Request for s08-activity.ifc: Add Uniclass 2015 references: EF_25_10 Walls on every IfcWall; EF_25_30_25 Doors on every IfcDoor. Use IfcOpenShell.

First a look at what the model holds.

```python
import ifcopenshell

model = ifcopenshell.open("s08-activity.ifc")
print(model.schema)
print("classifications:", [c.Name for c in model.by_type("IfcClassification")])
for ifc_class in ("IfcDoor", "IfcRoof", "IfcStair", "IfcWall", "IfcWindow"):
    print(ifc_class, len(model.by_type(ifc_class)))
```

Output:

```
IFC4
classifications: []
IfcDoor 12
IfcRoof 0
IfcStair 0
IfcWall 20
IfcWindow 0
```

```python
import ifcopenshell
import ifcopenshell.api.classification

model = ifcopenshell.open("s08-activity.ifc")

system = ifcopenshell.api.classification.add_classification(model, classification="Uniclass 2015")

codes = {
    "IfcWall": ("EF_25_10", "Walls"),
    "IfcDoor": ("EF_25_30_25", "Doors"),
}
for ifc_class, (code, name) in codes.items():
    products = model.by_type(ifc_class)
    ifcopenshell.api.classification.add_reference(
        model, products=products, classification=system, identification=code, name=name
    )
    print(code, len(products))

model.write("s08-activity-out.ifc")
```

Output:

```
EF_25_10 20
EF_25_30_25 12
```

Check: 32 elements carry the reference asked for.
